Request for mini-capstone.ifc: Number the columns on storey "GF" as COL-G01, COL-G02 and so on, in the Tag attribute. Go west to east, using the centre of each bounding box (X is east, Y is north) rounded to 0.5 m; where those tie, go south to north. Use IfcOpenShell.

First a look at what the model holds.

```python
import ifcopenshell
import ifcopenshell.util.element
import ifcopenshell.util.placement

model = ifcopenshell.open("mini-capstone.ifc")
print(model.schema)
storey = next(s for s in model.by_type("IfcBuildingStorey") if s.Name == "GF")
columns = [e for e in ifcopenshell.util.element.get_decomposition(storey) if e.is_a("IfcColumn")]
for e in sorted(columns, key=lambda e: e.id()):
    origin = ifcopenshell.util.placement.get_local_placement(e.ObjectPlacement)[:3, 3]
    print(e.id(), e.Tag, e.Name, origin.round(2) + 0.0, sep=" | ")
```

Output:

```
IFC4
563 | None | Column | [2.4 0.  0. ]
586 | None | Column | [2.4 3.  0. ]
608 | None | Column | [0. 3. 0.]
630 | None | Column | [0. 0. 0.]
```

```python
import ifcopenshell
import ifcopenshell.geom
import ifcopenshell.util.element
import ifcopenshell.util.shape

model = ifcopenshell.open("mini-capstone.ifc")
settings = ifcopenshell.geom.settings()
settings.set("use-world-coords", True)


def centre(element):
    shape = ifcopenshell.geom.create_shape(settings, element)
    return ifcopenshell.util.shape.get_bbox_centroid(shape.geometry)


storey = next(s for s in model.by_type("IfcBuildingStorey") if s.Name == "GF")
columns = [e for e in ifcopenshell.util.element.get_decomposition(storey) if e.is_a("IfcColumn")]

# Insertion points can sit at a corner or the storey origin, so sort by the geometry (in metres).
centres = {e: centre(e) for e in columns}
columns.sort(key=lambda e: (round(centres[e][0] / 0.5), centres[e][1]))

for i, e in enumerate(columns, start=1):
    number = f"COL-G{i:02d}"
    e.Tag = number
    print(e.id(), number)

model.write("mini-capstone_edited.ifc")
```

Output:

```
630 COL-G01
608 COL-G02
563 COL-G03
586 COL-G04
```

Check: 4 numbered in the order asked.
